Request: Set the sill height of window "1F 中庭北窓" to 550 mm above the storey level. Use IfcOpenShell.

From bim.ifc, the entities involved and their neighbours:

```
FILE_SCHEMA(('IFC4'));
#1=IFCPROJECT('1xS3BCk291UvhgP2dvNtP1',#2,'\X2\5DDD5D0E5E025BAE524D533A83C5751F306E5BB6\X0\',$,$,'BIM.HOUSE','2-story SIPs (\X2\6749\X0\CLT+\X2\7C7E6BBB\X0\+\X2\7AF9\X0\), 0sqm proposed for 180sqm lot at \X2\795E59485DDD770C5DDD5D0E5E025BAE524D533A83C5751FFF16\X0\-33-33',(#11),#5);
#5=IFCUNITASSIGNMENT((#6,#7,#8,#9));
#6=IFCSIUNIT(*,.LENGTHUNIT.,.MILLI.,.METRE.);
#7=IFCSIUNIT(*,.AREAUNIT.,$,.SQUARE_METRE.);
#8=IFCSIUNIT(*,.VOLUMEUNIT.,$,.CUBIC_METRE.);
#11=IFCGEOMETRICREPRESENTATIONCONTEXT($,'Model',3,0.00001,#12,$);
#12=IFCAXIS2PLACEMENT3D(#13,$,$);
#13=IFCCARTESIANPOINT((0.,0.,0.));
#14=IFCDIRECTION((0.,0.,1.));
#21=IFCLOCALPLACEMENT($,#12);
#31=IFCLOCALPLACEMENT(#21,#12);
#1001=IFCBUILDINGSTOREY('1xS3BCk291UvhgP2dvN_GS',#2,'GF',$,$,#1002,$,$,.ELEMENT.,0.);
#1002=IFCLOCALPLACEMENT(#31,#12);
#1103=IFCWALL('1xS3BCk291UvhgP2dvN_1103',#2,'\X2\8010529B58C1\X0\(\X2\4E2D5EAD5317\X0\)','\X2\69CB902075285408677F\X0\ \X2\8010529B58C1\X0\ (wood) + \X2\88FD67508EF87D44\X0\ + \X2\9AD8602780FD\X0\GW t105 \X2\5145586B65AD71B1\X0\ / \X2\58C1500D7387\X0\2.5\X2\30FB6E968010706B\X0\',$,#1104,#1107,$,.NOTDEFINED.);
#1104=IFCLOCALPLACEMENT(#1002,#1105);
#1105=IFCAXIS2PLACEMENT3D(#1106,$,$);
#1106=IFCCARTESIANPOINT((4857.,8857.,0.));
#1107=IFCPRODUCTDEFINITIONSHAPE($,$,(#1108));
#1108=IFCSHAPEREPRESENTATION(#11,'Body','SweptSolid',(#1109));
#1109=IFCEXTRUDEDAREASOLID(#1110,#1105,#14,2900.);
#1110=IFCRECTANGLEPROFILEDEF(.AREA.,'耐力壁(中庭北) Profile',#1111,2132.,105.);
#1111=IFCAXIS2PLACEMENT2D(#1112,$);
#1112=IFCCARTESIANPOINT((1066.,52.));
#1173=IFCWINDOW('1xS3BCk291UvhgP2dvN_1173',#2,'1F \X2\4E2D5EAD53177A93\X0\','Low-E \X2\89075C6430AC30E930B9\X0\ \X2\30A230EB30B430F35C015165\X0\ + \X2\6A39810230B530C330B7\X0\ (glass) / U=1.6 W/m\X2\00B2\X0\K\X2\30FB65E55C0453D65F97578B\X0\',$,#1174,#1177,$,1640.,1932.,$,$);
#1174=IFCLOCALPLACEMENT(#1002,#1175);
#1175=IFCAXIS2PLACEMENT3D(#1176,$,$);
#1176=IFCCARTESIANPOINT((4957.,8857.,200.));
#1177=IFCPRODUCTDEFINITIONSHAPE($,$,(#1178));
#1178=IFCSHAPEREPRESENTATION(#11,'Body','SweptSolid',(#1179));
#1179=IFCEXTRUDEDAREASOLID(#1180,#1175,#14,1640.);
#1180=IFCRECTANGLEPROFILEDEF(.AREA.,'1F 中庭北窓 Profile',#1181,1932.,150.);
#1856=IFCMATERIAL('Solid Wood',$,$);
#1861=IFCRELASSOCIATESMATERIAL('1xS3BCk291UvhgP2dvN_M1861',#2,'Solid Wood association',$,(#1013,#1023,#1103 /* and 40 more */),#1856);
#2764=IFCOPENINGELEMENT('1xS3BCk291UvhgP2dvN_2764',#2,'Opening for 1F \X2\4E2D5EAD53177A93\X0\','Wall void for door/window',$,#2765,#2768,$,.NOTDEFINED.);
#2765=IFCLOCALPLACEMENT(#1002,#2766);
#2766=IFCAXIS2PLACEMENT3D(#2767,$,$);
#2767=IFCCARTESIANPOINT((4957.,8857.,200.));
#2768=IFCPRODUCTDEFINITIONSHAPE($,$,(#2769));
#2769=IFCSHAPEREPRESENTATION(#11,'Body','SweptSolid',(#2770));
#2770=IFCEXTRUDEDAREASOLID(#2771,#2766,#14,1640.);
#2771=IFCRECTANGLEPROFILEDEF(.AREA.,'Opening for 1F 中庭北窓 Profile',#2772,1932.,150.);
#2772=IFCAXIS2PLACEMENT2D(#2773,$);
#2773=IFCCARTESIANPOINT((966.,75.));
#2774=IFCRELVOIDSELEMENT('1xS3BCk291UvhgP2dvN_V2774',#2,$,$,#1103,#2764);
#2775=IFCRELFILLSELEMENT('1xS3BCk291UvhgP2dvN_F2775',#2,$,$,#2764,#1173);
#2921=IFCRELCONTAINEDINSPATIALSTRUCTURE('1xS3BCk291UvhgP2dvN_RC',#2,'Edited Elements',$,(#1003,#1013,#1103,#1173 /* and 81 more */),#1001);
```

```python
import numpy as np
import ifcopenshell
import ifcopenshell.api.geometry
import ifcopenshell.geom
import ifcopenshell.util.element
import ifcopenshell.util.placement
import ifcopenshell.util.shape
import ifcopenshell.util.unit

model = ifcopenshell.open("bim.ifc")
unit_scale = ifcopenshell.util.unit.calculate_unit_scale(model)

window = model.by_guid("1xS3BCk291UvhgP2dvN_1173")
opening = window.FillsVoids[0].RelatingOpeningElement
storey = ifcopenshell.util.element.get_container(window, ifc_class="IfcBuildingStorey")
level = ifcopenshell.util.placement.get_local_placement(storey.ObjectPlacement)[2, 3]

# The opening's origin need not be at the sill, so measure its lowest point.
shape = ifcopenshell.geom.create_shape(ifcopenshell.geom.settings(), opening)
bottom = ifcopenshell.util.shape.get_shape_bottom_elevation(shape, shape.geometry) / unit_scale
dz = level + 0.55 / unit_scale - bottom

shift = np.array([0.0, 0.0, dz])
# The window is not placed relative to its opening, so move both.
for product in (opening, window):
    matrix = ifcopenshell.util.placement.get_local_placement(product.ObjectPlacement)
    matrix[:3, 3] += shift
    ifcopenshell.api.geometry.edit_object_placement(model, product=product, matrix=matrix, is_si=False)

print(f"moved by {dz * unit_scale:+.3f} m")

model.write("bim_rev.ifc")
```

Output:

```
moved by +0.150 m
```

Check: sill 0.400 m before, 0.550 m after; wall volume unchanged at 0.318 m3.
